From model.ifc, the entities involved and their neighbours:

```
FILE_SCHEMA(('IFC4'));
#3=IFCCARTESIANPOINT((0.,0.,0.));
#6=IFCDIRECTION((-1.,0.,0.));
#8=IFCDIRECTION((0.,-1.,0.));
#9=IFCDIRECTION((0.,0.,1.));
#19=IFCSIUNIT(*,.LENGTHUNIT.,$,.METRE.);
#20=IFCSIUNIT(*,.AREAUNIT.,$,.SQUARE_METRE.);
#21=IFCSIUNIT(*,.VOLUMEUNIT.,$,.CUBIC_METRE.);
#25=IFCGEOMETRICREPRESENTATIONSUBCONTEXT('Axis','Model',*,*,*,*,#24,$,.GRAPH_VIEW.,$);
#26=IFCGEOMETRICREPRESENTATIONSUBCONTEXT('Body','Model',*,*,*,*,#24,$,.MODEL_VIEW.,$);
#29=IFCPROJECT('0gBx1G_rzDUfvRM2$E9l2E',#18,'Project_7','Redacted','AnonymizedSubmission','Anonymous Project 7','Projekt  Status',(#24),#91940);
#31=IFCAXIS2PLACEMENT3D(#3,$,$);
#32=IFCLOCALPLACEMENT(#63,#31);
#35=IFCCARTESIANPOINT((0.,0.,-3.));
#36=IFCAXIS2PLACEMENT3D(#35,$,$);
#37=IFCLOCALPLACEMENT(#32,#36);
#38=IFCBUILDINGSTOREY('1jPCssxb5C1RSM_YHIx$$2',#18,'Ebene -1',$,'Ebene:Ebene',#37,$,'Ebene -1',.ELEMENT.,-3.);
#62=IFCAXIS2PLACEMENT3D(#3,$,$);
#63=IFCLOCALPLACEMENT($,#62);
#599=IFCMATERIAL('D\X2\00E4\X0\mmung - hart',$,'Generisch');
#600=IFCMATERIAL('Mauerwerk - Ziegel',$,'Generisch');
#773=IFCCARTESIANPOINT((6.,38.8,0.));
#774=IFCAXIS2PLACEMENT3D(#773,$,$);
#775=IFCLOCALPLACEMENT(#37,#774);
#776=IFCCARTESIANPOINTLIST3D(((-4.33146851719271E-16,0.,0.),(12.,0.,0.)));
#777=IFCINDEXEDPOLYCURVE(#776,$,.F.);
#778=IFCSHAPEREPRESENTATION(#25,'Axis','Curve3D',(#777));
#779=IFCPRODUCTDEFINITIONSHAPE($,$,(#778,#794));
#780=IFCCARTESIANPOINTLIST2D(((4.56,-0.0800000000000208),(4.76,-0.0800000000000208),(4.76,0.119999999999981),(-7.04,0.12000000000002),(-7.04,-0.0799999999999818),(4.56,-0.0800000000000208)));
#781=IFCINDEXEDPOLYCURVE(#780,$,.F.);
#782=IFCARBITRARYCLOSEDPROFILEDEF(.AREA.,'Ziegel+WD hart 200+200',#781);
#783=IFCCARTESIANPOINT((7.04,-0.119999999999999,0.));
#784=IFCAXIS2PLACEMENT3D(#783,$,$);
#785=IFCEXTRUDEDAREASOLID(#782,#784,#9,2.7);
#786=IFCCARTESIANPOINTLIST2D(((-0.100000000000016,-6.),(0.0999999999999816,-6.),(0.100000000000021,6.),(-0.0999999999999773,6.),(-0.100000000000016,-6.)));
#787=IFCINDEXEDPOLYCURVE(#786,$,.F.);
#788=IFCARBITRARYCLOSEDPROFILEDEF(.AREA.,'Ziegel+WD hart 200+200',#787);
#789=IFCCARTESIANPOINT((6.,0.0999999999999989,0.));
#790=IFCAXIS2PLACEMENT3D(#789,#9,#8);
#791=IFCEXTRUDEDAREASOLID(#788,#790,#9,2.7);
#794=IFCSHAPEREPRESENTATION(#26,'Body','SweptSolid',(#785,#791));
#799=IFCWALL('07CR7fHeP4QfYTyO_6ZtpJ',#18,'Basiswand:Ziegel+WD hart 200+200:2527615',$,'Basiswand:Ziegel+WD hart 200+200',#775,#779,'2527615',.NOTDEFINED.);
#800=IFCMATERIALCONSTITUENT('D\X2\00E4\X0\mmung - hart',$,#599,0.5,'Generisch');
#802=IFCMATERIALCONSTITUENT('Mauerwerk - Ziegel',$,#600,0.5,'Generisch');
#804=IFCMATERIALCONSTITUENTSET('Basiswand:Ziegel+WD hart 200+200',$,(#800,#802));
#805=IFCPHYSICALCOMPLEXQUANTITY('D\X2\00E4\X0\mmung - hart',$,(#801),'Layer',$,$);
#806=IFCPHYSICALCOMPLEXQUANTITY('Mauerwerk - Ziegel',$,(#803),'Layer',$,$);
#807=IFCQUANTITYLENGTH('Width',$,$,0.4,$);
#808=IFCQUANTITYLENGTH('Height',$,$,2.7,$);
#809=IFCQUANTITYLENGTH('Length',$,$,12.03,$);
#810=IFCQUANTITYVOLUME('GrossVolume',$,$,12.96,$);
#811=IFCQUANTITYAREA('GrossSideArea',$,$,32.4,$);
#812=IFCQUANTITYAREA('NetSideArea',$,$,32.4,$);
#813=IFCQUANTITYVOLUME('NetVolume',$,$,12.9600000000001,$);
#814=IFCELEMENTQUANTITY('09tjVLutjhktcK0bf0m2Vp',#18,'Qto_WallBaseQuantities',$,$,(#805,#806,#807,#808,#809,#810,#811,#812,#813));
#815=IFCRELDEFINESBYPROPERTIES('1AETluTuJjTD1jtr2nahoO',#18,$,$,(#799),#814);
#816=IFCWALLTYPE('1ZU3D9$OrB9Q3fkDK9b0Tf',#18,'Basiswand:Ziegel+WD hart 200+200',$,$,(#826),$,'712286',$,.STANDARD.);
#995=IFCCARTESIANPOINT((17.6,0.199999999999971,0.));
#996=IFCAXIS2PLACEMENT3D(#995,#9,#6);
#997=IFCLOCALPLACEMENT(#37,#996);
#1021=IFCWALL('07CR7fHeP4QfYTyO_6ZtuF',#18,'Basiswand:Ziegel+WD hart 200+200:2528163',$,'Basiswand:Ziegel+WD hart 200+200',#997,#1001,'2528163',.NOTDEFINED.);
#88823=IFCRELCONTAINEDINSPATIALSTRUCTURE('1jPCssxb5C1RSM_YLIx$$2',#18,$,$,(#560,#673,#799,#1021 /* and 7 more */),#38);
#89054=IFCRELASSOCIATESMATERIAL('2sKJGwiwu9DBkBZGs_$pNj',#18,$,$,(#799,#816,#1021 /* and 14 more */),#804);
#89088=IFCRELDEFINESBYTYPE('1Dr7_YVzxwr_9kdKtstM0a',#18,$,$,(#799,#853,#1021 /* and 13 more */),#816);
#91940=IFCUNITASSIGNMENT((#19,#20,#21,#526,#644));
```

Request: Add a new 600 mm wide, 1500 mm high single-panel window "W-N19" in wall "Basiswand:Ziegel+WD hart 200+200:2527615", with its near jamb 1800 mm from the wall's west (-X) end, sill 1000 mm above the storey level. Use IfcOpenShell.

```python
import numpy as np
import ifcopenshell
import ifcopenshell.api.feature
import ifcopenshell.api.geometry
import ifcopenshell.api.pset
import ifcopenshell.api.root
import ifcopenshell.api.spatial
import ifcopenshell.geom
import ifcopenshell.util.element
import ifcopenshell.util.placement
import ifcopenshell.util.representation
import ifcopenshell.util.shape
import ifcopenshell.util.unit

model = ifcopenshell.open("model.ifc")
unit_scale = ifcopenshell.util.unit.calculate_unit_scale(model)
area_scale = ifcopenshell.util.unit.calculate_unit_scale(model, "AREAUNIT")
volume_scale = ifcopenshell.util.unit.calculate_unit_scale(model, "VOLUMEUNIT")
settings = ifcopenshell.geom.settings()


def volume(element):
    """Net volume in cubic metres, openings subtracted."""
    shape = ifcopenshell.geom.create_shape(settings, element)
    return ifcopenshell.util.shape.get_volume(shape.geometry)


wall = model.by_guid("07CR7fHeP4QfYTyO_6ZtpJ")
storey = ifcopenshell.util.element.get_container(wall, ifc_class="IfcBuildingStorey")
context = ifcopenshell.util.representation.get_context(model, "Model", "Body", "MODEL_VIEW")
before = volume(wall)

width, height, from_end, sill = 0.6, 1.5, 1.8, 1  # metres

# The wall runs along its own X axis, and the end named is its -X end.
wall_shape = ifcopenshell.geom.create_shape(settings, wall)
x, y, z = ifcopenshell.util.shape.get_vertices(wall_shape.geometry).T
start = x.min() + from_end
face, thickness = float(y.min()), float(y.max() - y.min())
wall_matrix = ifcopenshell.util.placement.get_local_placement(wall.ObjectPlacement)
level = ifcopenshell.util.placement.get_local_placement(storey.ObjectPlacement)[2, 3]


def in_wall(x, y):
    """Placement at x, y metres in the wall's axes, at sill height."""
    matrix = wall_matrix.copy()
    matrix[:, 3] = wall_matrix @ np.array([x / unit_scale, y / unit_scale, 0.0, 1.0])
    matrix[2, 3] = level + sill / unit_scale
    return matrix


# Opening: a box that overshoots both wall faces by 50 mm.
opening = ifcopenshell.api.root.create_entity(model, ifc_class="IfcOpeningElement", predefined_type="OPENING")
box = ifcopenshell.api.geometry.add_wall_representation(
    model, context=context, length=width, height=height, thickness=thickness + 0.1
)
ifcopenshell.api.geometry.assign_representation(model, product=opening, representation=box)
ifcopenshell.api.geometry.edit_object_placement(model, product=opening, matrix=in_wall(start, face - 0.05), is_si=False)
ifcopenshell.api.feature.add_feature(model, feature=opening, element=wall)

window = ifcopenshell.api.root.create_entity(model, ifc_class="IfcWindow", name="W-N19", predefined_type="WINDOW")
window.OverallWidth, window.OverallHeight = width / unit_scale, height / unit_scale
window.PartitioningType = "SINGLE_PANEL"
body = ifcopenshell.api.geometry.add_window_representation(
    model,
    context=context,
    overall_width=window.OverallWidth,
    overall_height=window.OverallHeight,
    partition_type="SINGLE_PANEL",
)
ifcopenshell.api.geometry.assign_representation(model, product=window, representation=body)
ifcopenshell.api.spatial.assign_container(model, products=[window], relating_structure=storey)
ifcopenshell.api.feature.add_filling(model, opening=opening, element=window)

# Centre the window in the wall's thickness.
ifcopenshell.api.geometry.edit_object_placement(model, product=window, matrix=in_wall(start, face), is_si=False)
window_shape = ifcopenshell.geom.create_shape(settings, window)
depth = ifcopenshell.util.shape.get_vertices(window_shape.geometry)[:, 1]
offset = face + thickness / 2 - (depth.min() + depth.max()) / 2
ifcopenshell.api.geometry.edit_object_placement(model, product=window, matrix=in_wall(start, offset), is_si=False)

after = volume(wall)

# Update the wall's stored quantities.
qto = model.by_id(ifcopenshell.util.element.get_pset(wall, "Qto_WallBaseQuantities", should_inherit=False)["id"])
ifcopenshell.api.pset.edit_qto(model, qto=qto, properties={
    "NetSideArea": after / thickness / area_scale,
    "NetVolume": after / volume_scale,
})

print(f"wall volume {before:.3f} -> {after:.3f} m3")

model.write("model_rev.ifc")
```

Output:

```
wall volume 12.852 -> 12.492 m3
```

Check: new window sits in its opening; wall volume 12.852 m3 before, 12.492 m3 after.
